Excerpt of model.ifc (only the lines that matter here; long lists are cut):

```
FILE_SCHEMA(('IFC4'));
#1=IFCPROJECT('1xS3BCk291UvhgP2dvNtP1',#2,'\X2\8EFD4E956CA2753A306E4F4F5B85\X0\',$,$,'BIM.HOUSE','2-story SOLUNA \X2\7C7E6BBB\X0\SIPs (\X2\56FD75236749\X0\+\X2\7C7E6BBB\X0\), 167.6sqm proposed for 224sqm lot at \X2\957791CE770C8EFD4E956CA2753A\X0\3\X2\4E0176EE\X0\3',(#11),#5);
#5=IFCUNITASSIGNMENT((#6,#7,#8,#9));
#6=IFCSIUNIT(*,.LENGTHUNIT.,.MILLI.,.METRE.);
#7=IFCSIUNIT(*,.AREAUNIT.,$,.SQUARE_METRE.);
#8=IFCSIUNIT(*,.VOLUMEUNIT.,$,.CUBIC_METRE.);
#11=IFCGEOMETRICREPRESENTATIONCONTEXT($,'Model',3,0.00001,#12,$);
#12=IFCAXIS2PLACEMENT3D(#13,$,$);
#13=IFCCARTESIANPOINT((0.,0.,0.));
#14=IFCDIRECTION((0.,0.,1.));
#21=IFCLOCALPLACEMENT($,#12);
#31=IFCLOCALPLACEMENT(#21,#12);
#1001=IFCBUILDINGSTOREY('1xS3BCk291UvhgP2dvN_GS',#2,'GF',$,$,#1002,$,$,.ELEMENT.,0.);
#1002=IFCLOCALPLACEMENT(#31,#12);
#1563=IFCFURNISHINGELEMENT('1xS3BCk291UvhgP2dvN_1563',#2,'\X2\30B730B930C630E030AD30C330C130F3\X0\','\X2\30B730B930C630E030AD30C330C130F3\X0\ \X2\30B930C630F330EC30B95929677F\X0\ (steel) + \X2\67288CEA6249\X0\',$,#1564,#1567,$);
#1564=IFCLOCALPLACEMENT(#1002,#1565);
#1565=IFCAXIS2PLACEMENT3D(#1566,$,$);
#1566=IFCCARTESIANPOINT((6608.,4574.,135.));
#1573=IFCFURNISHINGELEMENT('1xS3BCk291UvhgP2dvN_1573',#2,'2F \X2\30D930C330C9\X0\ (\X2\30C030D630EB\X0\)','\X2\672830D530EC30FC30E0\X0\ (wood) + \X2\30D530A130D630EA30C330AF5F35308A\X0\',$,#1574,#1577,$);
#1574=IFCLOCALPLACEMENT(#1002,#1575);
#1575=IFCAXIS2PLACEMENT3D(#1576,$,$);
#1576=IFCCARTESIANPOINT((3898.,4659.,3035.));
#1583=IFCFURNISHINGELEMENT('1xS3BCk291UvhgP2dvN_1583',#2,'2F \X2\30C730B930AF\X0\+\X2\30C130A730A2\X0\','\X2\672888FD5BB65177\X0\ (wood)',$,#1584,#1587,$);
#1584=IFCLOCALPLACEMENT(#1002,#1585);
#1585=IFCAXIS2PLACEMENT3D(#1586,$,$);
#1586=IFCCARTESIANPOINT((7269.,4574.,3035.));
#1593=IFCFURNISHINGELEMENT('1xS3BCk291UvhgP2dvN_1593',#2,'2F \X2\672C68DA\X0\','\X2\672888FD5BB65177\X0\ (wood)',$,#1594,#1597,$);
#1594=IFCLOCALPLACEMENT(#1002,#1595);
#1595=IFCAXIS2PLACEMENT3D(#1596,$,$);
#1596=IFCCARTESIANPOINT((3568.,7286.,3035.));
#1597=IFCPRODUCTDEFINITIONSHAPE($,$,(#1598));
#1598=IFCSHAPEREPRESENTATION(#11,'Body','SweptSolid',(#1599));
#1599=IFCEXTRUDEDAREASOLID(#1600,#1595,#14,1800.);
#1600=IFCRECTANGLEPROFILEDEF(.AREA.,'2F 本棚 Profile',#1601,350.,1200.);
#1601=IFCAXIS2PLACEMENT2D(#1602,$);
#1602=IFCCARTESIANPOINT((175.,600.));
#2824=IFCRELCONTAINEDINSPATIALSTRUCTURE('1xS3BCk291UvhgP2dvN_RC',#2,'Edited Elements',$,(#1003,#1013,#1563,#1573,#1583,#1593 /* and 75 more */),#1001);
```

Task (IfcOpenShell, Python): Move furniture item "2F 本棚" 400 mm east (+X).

```python
import ifcopenshell
import ifcopenshell.api.geometry
import ifcopenshell.util.placement
import ifcopenshell.util.unit

model = ifcopenshell.open("model.ifc")
unit_scale = ifcopenshell.util.unit.calculate_unit_scale(model)

item = model.by_id(1593)
matrix = ifcopenshell.util.placement.get_local_placement(item.ObjectPlacement)
matrix[0, 3] += 0.4 / unit_scale
ifcopenshell.api.geometry.edit_object_placement(model, product=item, matrix=matrix, is_si=False)

print(ifcopenshell.util.placement.get_local_placement(item.ObjectPlacement).round(3) + 0.0)

model.write("model_v2.ifc")
```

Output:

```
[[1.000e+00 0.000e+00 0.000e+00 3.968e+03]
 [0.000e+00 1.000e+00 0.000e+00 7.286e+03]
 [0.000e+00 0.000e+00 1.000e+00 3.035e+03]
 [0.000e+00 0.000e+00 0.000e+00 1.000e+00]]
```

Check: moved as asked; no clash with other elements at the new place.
